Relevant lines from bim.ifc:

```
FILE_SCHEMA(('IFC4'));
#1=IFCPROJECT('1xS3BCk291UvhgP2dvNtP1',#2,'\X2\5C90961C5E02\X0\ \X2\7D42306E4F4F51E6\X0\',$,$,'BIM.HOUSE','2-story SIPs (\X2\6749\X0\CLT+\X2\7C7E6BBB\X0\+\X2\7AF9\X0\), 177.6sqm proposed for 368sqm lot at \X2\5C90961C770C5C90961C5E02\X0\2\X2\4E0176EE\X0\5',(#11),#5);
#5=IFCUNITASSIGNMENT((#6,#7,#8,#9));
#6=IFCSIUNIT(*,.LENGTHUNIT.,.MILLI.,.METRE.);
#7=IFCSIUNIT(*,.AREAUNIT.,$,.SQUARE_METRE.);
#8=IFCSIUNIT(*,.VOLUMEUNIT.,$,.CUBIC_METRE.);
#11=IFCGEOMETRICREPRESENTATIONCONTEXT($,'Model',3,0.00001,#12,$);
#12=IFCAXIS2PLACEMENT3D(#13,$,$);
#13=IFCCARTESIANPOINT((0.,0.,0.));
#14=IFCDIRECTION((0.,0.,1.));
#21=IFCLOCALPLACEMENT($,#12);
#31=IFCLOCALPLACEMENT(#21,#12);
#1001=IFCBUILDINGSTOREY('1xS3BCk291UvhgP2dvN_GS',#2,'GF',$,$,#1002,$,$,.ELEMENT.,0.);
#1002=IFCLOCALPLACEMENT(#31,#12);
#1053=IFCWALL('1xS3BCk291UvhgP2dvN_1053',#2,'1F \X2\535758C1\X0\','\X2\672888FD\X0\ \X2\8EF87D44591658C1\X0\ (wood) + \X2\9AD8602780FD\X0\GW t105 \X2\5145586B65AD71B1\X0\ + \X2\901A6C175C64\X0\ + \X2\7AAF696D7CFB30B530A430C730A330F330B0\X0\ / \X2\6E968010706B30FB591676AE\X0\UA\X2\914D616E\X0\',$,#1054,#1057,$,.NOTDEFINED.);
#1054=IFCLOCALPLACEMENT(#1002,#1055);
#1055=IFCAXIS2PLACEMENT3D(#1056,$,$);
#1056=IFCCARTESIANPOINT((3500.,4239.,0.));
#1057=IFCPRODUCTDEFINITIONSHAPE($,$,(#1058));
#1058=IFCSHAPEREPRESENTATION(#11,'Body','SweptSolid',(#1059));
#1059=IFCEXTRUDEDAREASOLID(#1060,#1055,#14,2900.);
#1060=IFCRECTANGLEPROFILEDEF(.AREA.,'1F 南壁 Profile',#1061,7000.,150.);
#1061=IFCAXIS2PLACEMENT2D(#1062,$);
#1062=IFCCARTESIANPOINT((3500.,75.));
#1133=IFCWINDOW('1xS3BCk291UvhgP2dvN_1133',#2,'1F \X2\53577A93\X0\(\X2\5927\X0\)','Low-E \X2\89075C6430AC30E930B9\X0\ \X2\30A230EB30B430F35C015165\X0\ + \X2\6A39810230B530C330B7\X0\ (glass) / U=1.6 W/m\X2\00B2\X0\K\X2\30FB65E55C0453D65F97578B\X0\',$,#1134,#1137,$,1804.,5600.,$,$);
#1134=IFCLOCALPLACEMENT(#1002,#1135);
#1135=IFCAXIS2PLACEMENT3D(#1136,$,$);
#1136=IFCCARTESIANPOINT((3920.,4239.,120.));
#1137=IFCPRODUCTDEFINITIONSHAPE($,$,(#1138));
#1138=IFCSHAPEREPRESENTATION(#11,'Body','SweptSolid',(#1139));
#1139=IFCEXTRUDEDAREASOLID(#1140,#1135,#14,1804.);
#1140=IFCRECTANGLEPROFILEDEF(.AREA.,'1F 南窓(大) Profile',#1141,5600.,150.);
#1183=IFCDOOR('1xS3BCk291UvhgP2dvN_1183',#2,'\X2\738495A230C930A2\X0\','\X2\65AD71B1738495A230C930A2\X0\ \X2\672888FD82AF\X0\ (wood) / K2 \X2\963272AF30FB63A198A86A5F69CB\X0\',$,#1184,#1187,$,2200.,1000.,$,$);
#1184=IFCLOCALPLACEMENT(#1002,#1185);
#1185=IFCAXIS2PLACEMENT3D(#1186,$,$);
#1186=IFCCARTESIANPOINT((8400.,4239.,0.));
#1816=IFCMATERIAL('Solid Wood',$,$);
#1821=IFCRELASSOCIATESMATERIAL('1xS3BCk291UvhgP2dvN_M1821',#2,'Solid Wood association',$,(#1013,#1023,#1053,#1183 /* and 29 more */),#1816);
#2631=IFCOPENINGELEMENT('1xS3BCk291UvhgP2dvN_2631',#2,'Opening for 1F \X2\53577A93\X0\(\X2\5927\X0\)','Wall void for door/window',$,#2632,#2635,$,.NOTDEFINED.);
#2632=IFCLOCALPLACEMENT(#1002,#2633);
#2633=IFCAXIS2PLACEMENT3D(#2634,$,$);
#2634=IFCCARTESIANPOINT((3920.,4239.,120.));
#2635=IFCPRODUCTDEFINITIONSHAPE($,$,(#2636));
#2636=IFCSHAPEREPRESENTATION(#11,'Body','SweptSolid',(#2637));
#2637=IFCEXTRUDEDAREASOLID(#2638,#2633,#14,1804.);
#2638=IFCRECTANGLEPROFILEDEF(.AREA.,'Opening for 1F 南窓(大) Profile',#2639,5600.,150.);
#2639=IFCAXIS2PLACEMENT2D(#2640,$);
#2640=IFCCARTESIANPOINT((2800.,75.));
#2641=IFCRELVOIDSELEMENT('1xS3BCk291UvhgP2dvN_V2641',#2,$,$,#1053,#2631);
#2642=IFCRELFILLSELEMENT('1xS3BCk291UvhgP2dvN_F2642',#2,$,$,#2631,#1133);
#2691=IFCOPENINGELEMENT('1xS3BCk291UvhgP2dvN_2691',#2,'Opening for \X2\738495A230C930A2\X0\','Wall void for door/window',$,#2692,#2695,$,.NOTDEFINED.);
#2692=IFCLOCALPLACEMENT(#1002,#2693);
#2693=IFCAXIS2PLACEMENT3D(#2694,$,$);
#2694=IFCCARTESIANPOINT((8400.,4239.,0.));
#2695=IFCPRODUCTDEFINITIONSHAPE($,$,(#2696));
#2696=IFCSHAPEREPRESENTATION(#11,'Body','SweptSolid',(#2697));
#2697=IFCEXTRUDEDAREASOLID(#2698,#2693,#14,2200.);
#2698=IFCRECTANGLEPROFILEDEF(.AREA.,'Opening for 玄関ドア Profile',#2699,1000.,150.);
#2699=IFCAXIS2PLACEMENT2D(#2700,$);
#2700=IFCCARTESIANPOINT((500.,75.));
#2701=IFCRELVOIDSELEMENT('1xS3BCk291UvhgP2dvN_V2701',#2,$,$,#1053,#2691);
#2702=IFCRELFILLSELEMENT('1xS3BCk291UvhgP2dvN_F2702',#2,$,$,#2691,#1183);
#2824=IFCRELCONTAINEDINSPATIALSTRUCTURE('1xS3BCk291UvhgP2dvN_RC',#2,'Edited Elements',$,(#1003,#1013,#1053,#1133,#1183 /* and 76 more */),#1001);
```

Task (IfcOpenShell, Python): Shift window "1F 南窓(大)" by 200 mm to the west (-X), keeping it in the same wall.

```python
import ifcopenshell
import ifcopenshell.api.geometry
import ifcopenshell.util.placement

model = ifcopenshell.open("bim.ifc")

window = model.by_guid("1xS3BCk291UvhgP2dvN_1133")
opening = window.FillsVoids[0].RelatingOpeningElement
wall = opening.VoidsElements[0].RelatingBuildingElement

wall_matrix = ifcopenshell.util.placement.get_local_placement(wall.ObjectPlacement)
shift = wall_matrix[:3, 0] * -200.0
before = ifcopenshell.util.placement.get_local_placement(window.ObjectPlacement)[:3, 3].copy()

# The window is not placed relative to its opening, so move both.
for product in (opening, window):
    matrix = ifcopenshell.util.placement.get_local_placement(product.ObjectPlacement)
    matrix[:3, 3] += shift
    ifcopenshell.api.geometry.edit_object_placement(model, product=product, matrix=matrix, is_si=False)

after = ifcopenshell.util.placement.get_local_placement(window.ObjectPlacement)[:3, 3]
print("window moved by", (after - before).round(3) + 0.0)

model.write("bim-out.ifc")
```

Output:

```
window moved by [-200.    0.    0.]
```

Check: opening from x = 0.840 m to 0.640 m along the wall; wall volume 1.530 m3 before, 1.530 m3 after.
